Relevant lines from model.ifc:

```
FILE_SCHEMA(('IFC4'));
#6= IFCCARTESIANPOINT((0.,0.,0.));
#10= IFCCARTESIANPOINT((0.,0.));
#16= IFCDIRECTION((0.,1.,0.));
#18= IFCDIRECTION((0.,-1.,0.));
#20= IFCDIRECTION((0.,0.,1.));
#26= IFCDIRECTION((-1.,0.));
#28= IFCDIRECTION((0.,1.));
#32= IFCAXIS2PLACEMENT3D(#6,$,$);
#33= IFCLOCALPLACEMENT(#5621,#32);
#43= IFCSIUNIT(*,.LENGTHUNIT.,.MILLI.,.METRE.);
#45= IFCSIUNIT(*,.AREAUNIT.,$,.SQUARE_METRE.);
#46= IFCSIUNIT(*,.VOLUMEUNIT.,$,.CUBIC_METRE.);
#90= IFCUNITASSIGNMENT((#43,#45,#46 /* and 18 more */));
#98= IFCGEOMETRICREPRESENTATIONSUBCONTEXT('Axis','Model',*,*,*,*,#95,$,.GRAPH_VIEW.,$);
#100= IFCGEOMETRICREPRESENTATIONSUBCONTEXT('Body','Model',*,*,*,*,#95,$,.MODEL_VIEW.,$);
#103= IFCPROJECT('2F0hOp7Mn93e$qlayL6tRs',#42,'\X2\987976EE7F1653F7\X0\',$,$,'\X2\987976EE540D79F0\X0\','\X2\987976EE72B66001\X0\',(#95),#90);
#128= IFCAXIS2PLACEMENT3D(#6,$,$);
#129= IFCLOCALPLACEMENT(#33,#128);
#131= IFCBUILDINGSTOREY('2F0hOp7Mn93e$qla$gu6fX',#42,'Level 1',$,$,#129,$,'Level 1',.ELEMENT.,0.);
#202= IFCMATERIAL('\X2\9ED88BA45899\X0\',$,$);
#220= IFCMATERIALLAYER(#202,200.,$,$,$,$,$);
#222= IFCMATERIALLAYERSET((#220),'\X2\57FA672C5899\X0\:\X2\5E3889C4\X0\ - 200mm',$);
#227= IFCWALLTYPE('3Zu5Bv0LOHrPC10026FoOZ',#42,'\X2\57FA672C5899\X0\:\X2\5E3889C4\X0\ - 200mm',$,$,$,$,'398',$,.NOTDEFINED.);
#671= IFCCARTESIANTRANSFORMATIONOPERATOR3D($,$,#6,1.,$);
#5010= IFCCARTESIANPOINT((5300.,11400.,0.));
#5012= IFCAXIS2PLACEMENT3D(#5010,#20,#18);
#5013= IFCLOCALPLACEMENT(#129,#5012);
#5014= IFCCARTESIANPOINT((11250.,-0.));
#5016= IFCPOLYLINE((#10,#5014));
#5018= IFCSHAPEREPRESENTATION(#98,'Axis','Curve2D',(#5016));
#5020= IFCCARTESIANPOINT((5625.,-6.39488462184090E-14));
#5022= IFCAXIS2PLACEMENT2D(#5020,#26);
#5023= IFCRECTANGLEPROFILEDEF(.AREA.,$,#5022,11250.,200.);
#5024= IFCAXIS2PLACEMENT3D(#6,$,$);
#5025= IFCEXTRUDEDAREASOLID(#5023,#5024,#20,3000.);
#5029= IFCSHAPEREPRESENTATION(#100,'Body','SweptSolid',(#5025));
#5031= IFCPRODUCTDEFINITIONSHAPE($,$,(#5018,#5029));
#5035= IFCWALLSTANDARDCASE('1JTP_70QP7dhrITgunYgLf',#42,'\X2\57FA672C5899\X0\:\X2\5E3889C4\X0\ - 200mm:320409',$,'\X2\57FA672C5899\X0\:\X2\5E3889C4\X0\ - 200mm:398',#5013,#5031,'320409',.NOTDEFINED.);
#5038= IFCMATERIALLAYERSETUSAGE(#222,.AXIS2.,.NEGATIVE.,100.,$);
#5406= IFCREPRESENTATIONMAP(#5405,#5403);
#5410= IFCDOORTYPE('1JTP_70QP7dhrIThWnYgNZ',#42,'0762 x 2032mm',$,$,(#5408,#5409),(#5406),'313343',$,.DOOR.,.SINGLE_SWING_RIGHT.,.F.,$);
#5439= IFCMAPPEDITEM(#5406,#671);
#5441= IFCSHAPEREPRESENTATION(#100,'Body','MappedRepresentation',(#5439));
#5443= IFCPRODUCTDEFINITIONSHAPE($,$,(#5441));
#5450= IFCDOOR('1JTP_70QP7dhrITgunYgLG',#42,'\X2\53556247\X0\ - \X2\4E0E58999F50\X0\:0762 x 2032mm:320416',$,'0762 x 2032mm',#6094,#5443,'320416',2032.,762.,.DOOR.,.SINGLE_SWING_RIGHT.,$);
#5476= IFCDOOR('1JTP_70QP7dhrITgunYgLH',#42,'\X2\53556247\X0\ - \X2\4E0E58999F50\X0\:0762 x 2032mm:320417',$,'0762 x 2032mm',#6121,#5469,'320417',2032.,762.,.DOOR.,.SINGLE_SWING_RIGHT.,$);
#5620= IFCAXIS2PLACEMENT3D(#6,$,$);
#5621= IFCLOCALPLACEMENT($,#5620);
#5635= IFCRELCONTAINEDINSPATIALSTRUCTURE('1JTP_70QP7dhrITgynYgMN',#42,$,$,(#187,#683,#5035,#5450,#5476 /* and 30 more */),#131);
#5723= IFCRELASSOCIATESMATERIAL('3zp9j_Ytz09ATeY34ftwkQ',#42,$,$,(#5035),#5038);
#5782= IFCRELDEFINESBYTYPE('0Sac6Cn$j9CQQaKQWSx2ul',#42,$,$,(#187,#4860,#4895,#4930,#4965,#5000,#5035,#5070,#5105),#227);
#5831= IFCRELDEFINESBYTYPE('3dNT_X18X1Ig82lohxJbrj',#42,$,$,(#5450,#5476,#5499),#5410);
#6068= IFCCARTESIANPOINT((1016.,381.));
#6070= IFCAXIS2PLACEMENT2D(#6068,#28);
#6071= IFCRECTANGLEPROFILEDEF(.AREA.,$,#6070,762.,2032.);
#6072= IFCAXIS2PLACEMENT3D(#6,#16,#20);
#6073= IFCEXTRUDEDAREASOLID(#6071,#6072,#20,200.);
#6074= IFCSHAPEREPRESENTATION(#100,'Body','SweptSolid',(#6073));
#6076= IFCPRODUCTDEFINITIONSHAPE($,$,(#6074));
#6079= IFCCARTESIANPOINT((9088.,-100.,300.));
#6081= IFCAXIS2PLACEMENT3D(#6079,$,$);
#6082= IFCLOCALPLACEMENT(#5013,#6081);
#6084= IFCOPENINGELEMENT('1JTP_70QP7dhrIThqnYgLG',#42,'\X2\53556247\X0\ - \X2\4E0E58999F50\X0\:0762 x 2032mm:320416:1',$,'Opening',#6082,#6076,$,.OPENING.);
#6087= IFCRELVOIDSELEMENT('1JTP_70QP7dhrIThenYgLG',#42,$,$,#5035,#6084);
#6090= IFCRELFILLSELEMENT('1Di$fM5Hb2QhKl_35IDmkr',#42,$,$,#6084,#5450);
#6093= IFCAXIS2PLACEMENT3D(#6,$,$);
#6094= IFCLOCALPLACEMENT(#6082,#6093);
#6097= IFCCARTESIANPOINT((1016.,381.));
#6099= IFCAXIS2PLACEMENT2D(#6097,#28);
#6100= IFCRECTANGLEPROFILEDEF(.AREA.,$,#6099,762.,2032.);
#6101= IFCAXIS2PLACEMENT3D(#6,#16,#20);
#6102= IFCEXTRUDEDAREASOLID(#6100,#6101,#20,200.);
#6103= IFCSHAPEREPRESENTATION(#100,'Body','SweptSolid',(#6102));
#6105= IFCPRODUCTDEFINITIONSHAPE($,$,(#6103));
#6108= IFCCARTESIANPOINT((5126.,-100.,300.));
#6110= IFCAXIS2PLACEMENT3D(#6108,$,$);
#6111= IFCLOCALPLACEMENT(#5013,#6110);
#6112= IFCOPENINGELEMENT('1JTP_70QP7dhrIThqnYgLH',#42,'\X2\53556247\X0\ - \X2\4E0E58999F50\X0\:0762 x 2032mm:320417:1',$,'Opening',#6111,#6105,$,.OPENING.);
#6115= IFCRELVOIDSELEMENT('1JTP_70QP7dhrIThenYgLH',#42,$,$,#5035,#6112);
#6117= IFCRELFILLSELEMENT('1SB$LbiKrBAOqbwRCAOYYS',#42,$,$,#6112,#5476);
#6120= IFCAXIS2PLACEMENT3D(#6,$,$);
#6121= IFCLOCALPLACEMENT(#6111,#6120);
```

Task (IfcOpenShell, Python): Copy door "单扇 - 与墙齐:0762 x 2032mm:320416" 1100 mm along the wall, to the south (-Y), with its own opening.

```python
import ifcopenshell
import ifcopenshell.api.feature
import ifcopenshell.api.geometry
import ifcopenshell.api.root
import ifcopenshell.geom
import ifcopenshell.util.element
import ifcopenshell.util.placement
import ifcopenshell.util.shape
import ifcopenshell.util.unit

model = ifcopenshell.open("model.ifc")
unit_scale = ifcopenshell.util.unit.calculate_unit_scale(model)
settings = ifcopenshell.geom.settings()


def volume(element):
    """Net volume in cubic metres, openings subtracted."""
    shape = ifcopenshell.geom.create_shape(settings, element)
    return ifcopenshell.util.shape.get_volume(shape.geometry)


def reuse_history(source, copy):
    """copy_class also copies each property set's owner history, people and application; keep the originals."""
    for rel in copy.IsDefinedBy:
        if rel.is_a("IfcRelDefinesByProperties") and (history := rel.RelatingPropertyDefinition.OwnerHistory):
            rel.RelatingPropertyDefinition.OwnerHistory = source.OwnerHistory
            ifcopenshell.util.element.remove_deep2(model, history)


door = model.by_id(5450)
opening = door.FillsVoids[0].RelatingOpeningElement
wall = opening.VoidsElements[0].RelatingBuildingElement
before = volume(wall)
shift = ifcopenshell.util.placement.get_local_placement(wall.ObjectPlacement)[:3, 0] * 1.1 / unit_scale

# copy_class copies the void relationship, type, container and properties, but no geometry.
new_opening = ifcopenshell.api.root.copy_class(model, product=opening)
new_opening.Representation = ifcopenshell.util.element.copy_deep(
    model, opening.Representation, exclude=["IfcGeometricRepresentationContext", "IfcRepresentationMap"]
)
new_opening.Name = "单扇 - 与墙齐:0762 x 2032mm"
new_door = ifcopenshell.api.root.copy_class(model, product=door)
new_door.Representation = ifcopenshell.util.element.copy_deep(
    model, door.Representation, exclude=["IfcGeometricRepresentationContext", "IfcRepresentationMap"]
)
new_door.Name = "单扇 - 与墙齐:0762 x 2032mm"
new_door.Tag = None
reuse_history(door, new_door)
ifcopenshell.api.feature.add_filling(model, opening=new_opening, element=new_door)

for old, new in ((opening, new_opening), (door, new_door)):
    matrix = ifcopenshell.util.placement.get_local_placement(old.ObjectPlacement)
    matrix[:3, 3] += shift
    ifcopenshell.api.geometry.edit_object_placement(model, product=new, matrix=matrix, is_si=False)

after = volume(wall)

print(f"wall volume {before:.3f} -> {after:.3f} m3")

model.write("model_rev.ifc")
```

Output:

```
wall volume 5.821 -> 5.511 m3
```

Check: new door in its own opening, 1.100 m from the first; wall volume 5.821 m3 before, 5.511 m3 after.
